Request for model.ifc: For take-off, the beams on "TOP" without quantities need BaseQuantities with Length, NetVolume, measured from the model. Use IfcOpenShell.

First a look at what the model holds.

```python
import ifcopenshell
import ifcopenshell.util.element
import ifcopenshell.util.unit

model = ifcopenshell.open("model.ifc")
print(model.schema)
for unit_type in ("LENGTHUNIT", "AREAUNIT", "VOLUMEUNIT"):
    print(unit_type, ifcopenshell.util.unit.calculate_unit_scale(model, unit_type))
storey = next(s for s in model.by_type("IfcBuildingStorey") if s.Name == "TOP")
beams = [e for e in ifcopenshell.util.element.get_decomposition(storey) if e.is_a("IfcBeam")]
for e in sorted(beams, key=lambda e: e.id()):
    print(e.id(), e.is_a(), e.Name, list(ifcopenshell.util.element.get_psets(e, qtos_only=True)), sep=" | ")
```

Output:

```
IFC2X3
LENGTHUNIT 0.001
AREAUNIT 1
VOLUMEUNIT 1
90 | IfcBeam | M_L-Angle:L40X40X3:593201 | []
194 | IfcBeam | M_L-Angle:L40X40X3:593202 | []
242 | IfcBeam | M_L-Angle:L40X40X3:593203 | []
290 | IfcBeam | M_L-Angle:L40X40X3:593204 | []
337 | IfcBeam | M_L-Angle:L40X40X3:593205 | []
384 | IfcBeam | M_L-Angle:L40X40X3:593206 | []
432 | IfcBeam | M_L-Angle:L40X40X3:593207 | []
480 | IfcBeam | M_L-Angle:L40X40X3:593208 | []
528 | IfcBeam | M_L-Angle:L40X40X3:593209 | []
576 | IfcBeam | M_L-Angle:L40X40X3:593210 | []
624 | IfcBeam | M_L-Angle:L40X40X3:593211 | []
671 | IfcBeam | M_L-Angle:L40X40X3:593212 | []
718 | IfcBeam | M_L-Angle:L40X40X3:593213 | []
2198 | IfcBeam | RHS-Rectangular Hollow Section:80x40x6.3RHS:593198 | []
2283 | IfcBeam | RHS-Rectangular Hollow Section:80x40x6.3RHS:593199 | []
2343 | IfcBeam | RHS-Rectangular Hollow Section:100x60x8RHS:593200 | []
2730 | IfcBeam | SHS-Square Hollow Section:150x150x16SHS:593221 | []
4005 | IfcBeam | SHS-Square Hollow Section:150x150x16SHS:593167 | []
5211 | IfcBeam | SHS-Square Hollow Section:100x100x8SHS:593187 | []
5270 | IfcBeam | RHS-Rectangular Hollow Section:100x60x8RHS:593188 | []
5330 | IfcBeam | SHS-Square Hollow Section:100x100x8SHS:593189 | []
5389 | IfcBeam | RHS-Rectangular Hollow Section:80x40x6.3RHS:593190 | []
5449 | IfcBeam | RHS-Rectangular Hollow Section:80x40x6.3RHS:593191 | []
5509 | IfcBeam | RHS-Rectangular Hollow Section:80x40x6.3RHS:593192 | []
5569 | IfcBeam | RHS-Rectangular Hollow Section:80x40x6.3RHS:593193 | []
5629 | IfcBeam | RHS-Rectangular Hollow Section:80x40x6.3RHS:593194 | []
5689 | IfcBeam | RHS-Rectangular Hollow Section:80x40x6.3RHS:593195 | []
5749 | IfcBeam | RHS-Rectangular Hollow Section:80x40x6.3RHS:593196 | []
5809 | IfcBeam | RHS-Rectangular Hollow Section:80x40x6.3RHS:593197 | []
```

```python
import ifcopenshell
import ifcopenshell.api.pset
import ifcopenshell.geom
import ifcopenshell.util.element
import ifcopenshell.util.shape
import ifcopenshell.util.unit

model = ifcopenshell.open("model.ifc")
unit_scale = ifcopenshell.util.unit.calculate_unit_scale(model)
volume_scale = ifcopenshell.util.unit.calculate_unit_scale(model, "VOLUMEUNIT")
settings = ifcopenshell.geom.settings()

storey = next(s for s in model.by_type("IfcBuildingStorey") if s.Name == "TOP")
beams = [e for e in ifcopenshell.util.element.get_decomposition(storey) if e.is_a("IfcBeam")]

for e in sorted(beams, key=lambda e: e.id()):
    if ifcopenshell.util.element.get_psets(e, qtos_only=True, should_inherit=False):
        continue
    # Geometry comes back in metres, in the element's own axes.
    shape = ifcopenshell.geom.create_shape(settings, e)
    values = {
        "Length": ifcopenshell.util.shape.get_max_xyz(shape.geometry) / unit_scale,
        "NetVolume": ifcopenshell.util.shape.get_volume(shape.geometry) / volume_scale,
    }
    qto = ifcopenshell.api.pset.add_qto(model, product=e, name="BaseQuantities")
    ifcopenshell.api.pset.edit_qto(model, qto=qto, properties=values)
    print(e.id(), {k: round(v, 3) for k, v in values.items()})

model.write("model-out.ifc")
```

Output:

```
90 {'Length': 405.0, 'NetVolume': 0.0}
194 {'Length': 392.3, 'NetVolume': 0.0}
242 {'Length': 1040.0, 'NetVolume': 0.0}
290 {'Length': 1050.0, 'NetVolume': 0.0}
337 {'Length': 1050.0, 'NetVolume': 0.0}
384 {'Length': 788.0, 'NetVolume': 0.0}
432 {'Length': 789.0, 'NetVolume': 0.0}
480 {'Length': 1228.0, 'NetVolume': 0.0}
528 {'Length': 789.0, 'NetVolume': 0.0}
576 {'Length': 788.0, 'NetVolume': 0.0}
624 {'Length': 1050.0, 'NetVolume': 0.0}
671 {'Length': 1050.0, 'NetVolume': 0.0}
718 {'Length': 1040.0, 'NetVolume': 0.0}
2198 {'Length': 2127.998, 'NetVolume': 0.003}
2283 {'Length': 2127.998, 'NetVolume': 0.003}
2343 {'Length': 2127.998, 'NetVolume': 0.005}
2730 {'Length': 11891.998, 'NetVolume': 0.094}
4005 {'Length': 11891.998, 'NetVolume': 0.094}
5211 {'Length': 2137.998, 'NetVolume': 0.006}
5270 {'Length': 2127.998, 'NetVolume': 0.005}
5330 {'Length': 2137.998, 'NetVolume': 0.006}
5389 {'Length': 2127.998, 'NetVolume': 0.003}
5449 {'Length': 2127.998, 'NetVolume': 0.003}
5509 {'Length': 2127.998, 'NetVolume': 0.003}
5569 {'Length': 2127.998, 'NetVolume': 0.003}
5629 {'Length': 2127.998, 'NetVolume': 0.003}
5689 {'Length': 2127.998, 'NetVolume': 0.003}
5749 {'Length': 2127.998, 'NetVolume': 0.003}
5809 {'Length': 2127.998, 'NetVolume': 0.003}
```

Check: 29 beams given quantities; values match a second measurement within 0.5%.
